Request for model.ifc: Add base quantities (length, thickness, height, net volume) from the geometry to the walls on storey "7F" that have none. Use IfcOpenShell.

First a look at what the model holds.

```python
import ifcopenshell
import ifcopenshell.util.element
import ifcopenshell.util.unit

model = ifcopenshell.open("model.ifc")
print(model.schema)
for unit_type in ("LENGTHUNIT", "AREAUNIT", "VOLUMEUNIT"):
    print(unit_type, ifcopenshell.util.unit.calculate_unit_scale(model, unit_type))
storey = next(s for s in model.by_type("IfcBuildingStorey") if s.Name == "7F")
walls = [e for e in ifcopenshell.util.element.get_decomposition(storey) if e.is_a("IfcWall")]
for e in sorted(walls, key=lambda e: e.id()):
    print(e.id(), e.is_a(), e.Name, list(ifcopenshell.util.element.get_psets(e, qtos_only=True)), sep=" | ")
```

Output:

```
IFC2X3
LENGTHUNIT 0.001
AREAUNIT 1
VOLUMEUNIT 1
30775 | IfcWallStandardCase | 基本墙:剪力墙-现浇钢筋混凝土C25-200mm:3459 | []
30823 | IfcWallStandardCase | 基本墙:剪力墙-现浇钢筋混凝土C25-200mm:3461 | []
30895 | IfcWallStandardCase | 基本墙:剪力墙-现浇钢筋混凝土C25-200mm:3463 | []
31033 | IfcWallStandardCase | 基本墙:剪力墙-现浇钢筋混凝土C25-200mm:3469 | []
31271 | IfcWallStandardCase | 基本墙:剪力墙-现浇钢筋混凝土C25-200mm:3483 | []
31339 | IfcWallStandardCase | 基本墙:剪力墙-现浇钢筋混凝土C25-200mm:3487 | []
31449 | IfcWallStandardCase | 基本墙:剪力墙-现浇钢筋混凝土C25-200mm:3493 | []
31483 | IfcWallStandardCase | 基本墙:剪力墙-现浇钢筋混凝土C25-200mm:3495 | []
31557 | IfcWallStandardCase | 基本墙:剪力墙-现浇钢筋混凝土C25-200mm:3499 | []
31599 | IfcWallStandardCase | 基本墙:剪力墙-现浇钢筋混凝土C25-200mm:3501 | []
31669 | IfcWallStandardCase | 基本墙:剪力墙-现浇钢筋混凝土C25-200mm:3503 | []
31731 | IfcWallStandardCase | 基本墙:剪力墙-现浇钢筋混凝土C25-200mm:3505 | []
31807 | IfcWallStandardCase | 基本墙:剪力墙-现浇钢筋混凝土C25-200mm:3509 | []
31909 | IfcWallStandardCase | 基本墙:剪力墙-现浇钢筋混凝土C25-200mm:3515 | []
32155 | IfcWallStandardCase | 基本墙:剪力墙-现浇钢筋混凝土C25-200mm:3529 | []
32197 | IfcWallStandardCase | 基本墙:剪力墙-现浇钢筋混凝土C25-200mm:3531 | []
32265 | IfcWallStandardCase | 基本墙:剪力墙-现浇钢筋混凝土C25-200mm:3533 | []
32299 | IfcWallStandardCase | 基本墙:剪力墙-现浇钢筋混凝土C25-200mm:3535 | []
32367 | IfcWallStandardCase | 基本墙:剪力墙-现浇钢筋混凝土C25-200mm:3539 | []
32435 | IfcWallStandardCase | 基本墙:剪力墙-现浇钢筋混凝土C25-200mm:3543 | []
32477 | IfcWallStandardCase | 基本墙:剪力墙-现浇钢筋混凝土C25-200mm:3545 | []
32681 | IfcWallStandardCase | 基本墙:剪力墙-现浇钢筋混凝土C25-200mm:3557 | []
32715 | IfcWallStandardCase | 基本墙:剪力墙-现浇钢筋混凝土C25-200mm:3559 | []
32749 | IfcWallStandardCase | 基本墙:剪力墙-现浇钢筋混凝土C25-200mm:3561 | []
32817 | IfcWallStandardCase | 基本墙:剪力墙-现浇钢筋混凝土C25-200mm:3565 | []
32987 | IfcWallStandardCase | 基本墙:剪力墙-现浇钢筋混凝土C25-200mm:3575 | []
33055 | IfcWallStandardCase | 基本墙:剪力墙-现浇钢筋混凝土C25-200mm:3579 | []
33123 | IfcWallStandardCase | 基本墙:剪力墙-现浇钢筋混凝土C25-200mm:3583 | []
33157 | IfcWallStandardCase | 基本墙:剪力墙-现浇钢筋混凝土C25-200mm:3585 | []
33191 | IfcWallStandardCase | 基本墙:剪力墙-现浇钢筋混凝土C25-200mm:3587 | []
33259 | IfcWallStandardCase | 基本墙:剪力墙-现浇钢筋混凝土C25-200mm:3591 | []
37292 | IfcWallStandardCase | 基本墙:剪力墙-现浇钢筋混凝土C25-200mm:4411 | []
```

```python
import ifcopenshell
import ifcopenshell.api.pset
import ifcopenshell.geom
import ifcopenshell.util.element
import ifcopenshell.util.shape
import ifcopenshell.util.unit

model = ifcopenshell.open("model.ifc")
unit_scale = ifcopenshell.util.unit.calculate_unit_scale(model)
volume_scale = ifcopenshell.util.unit.calculate_unit_scale(model, "VOLUMEUNIT")
settings = ifcopenshell.geom.settings()

storey = next(s for s in model.by_type("IfcBuildingStorey") if s.Name == "7F")
walls = [e for e in ifcopenshell.util.element.get_decomposition(storey) if e.is_a("IfcWall")]

for e in sorted(walls, key=lambda e: e.id()):
    if ifcopenshell.util.element.get_psets(e, qtos_only=True, should_inherit=False):
        continue
    # Geometry comes back in metres, in the element's own axes.
    shape = ifcopenshell.geom.create_shape(settings, e)
    values = {
        "Length": ifcopenshell.util.shape.get_x(shape.geometry) / unit_scale,
        "Width": ifcopenshell.util.shape.get_y(shape.geometry) / unit_scale,
        "Height": ifcopenshell.util.shape.get_z(shape.geometry) / unit_scale,
        "NetVolume": ifcopenshell.util.shape.get_volume(shape.geometry) / volume_scale,
    }
    qto = ifcopenshell.api.pset.add_qto(model, product=e, name="BaseQuantities")
    ifcopenshell.api.pset.edit_qto(model, qto=qto, properties=values)
    print(e.id(), {k: round(v, 3) for k, v in values.items()})

model.write("model_rev.ifc")
```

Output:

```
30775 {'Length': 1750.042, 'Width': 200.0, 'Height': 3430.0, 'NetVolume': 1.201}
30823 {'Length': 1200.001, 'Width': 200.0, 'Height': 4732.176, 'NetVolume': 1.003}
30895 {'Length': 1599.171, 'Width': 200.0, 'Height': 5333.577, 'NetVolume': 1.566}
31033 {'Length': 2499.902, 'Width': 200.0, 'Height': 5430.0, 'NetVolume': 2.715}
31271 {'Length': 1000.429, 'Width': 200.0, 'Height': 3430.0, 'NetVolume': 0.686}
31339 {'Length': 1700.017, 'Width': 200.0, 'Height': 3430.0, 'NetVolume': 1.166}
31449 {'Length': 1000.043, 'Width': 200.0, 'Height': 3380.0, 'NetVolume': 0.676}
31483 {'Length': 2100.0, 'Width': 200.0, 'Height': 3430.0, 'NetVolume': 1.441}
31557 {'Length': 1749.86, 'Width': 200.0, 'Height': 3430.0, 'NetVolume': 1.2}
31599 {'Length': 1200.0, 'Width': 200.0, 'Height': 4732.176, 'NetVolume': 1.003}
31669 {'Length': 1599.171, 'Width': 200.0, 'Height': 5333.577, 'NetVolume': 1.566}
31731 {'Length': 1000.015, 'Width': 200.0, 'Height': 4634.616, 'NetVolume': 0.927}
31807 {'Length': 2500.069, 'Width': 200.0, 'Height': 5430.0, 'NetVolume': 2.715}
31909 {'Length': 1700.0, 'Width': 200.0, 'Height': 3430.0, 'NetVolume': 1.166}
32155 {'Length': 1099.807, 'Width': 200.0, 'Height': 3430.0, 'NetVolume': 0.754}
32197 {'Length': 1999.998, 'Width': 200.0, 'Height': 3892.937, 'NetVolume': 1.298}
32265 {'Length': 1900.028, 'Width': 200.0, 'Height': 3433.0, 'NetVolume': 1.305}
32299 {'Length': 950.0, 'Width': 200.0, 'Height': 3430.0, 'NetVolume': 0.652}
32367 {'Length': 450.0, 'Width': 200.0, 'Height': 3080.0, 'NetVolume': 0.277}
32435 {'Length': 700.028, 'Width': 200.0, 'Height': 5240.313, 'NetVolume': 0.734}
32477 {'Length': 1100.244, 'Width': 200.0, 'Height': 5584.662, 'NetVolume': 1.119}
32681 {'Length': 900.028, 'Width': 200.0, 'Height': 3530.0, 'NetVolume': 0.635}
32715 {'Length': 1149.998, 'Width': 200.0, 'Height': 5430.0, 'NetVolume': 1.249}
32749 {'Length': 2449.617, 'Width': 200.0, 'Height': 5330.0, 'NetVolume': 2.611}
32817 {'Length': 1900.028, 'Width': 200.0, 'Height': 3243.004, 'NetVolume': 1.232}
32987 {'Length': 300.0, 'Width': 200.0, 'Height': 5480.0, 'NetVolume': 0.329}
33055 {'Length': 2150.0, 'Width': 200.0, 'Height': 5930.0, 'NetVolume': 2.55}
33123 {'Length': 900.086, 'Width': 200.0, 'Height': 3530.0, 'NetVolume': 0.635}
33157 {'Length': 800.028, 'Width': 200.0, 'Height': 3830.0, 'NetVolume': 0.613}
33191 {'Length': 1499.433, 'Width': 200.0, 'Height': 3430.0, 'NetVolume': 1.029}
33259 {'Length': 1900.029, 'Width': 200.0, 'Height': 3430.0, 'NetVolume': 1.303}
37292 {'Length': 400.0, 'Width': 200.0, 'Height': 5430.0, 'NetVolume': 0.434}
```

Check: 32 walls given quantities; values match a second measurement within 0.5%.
